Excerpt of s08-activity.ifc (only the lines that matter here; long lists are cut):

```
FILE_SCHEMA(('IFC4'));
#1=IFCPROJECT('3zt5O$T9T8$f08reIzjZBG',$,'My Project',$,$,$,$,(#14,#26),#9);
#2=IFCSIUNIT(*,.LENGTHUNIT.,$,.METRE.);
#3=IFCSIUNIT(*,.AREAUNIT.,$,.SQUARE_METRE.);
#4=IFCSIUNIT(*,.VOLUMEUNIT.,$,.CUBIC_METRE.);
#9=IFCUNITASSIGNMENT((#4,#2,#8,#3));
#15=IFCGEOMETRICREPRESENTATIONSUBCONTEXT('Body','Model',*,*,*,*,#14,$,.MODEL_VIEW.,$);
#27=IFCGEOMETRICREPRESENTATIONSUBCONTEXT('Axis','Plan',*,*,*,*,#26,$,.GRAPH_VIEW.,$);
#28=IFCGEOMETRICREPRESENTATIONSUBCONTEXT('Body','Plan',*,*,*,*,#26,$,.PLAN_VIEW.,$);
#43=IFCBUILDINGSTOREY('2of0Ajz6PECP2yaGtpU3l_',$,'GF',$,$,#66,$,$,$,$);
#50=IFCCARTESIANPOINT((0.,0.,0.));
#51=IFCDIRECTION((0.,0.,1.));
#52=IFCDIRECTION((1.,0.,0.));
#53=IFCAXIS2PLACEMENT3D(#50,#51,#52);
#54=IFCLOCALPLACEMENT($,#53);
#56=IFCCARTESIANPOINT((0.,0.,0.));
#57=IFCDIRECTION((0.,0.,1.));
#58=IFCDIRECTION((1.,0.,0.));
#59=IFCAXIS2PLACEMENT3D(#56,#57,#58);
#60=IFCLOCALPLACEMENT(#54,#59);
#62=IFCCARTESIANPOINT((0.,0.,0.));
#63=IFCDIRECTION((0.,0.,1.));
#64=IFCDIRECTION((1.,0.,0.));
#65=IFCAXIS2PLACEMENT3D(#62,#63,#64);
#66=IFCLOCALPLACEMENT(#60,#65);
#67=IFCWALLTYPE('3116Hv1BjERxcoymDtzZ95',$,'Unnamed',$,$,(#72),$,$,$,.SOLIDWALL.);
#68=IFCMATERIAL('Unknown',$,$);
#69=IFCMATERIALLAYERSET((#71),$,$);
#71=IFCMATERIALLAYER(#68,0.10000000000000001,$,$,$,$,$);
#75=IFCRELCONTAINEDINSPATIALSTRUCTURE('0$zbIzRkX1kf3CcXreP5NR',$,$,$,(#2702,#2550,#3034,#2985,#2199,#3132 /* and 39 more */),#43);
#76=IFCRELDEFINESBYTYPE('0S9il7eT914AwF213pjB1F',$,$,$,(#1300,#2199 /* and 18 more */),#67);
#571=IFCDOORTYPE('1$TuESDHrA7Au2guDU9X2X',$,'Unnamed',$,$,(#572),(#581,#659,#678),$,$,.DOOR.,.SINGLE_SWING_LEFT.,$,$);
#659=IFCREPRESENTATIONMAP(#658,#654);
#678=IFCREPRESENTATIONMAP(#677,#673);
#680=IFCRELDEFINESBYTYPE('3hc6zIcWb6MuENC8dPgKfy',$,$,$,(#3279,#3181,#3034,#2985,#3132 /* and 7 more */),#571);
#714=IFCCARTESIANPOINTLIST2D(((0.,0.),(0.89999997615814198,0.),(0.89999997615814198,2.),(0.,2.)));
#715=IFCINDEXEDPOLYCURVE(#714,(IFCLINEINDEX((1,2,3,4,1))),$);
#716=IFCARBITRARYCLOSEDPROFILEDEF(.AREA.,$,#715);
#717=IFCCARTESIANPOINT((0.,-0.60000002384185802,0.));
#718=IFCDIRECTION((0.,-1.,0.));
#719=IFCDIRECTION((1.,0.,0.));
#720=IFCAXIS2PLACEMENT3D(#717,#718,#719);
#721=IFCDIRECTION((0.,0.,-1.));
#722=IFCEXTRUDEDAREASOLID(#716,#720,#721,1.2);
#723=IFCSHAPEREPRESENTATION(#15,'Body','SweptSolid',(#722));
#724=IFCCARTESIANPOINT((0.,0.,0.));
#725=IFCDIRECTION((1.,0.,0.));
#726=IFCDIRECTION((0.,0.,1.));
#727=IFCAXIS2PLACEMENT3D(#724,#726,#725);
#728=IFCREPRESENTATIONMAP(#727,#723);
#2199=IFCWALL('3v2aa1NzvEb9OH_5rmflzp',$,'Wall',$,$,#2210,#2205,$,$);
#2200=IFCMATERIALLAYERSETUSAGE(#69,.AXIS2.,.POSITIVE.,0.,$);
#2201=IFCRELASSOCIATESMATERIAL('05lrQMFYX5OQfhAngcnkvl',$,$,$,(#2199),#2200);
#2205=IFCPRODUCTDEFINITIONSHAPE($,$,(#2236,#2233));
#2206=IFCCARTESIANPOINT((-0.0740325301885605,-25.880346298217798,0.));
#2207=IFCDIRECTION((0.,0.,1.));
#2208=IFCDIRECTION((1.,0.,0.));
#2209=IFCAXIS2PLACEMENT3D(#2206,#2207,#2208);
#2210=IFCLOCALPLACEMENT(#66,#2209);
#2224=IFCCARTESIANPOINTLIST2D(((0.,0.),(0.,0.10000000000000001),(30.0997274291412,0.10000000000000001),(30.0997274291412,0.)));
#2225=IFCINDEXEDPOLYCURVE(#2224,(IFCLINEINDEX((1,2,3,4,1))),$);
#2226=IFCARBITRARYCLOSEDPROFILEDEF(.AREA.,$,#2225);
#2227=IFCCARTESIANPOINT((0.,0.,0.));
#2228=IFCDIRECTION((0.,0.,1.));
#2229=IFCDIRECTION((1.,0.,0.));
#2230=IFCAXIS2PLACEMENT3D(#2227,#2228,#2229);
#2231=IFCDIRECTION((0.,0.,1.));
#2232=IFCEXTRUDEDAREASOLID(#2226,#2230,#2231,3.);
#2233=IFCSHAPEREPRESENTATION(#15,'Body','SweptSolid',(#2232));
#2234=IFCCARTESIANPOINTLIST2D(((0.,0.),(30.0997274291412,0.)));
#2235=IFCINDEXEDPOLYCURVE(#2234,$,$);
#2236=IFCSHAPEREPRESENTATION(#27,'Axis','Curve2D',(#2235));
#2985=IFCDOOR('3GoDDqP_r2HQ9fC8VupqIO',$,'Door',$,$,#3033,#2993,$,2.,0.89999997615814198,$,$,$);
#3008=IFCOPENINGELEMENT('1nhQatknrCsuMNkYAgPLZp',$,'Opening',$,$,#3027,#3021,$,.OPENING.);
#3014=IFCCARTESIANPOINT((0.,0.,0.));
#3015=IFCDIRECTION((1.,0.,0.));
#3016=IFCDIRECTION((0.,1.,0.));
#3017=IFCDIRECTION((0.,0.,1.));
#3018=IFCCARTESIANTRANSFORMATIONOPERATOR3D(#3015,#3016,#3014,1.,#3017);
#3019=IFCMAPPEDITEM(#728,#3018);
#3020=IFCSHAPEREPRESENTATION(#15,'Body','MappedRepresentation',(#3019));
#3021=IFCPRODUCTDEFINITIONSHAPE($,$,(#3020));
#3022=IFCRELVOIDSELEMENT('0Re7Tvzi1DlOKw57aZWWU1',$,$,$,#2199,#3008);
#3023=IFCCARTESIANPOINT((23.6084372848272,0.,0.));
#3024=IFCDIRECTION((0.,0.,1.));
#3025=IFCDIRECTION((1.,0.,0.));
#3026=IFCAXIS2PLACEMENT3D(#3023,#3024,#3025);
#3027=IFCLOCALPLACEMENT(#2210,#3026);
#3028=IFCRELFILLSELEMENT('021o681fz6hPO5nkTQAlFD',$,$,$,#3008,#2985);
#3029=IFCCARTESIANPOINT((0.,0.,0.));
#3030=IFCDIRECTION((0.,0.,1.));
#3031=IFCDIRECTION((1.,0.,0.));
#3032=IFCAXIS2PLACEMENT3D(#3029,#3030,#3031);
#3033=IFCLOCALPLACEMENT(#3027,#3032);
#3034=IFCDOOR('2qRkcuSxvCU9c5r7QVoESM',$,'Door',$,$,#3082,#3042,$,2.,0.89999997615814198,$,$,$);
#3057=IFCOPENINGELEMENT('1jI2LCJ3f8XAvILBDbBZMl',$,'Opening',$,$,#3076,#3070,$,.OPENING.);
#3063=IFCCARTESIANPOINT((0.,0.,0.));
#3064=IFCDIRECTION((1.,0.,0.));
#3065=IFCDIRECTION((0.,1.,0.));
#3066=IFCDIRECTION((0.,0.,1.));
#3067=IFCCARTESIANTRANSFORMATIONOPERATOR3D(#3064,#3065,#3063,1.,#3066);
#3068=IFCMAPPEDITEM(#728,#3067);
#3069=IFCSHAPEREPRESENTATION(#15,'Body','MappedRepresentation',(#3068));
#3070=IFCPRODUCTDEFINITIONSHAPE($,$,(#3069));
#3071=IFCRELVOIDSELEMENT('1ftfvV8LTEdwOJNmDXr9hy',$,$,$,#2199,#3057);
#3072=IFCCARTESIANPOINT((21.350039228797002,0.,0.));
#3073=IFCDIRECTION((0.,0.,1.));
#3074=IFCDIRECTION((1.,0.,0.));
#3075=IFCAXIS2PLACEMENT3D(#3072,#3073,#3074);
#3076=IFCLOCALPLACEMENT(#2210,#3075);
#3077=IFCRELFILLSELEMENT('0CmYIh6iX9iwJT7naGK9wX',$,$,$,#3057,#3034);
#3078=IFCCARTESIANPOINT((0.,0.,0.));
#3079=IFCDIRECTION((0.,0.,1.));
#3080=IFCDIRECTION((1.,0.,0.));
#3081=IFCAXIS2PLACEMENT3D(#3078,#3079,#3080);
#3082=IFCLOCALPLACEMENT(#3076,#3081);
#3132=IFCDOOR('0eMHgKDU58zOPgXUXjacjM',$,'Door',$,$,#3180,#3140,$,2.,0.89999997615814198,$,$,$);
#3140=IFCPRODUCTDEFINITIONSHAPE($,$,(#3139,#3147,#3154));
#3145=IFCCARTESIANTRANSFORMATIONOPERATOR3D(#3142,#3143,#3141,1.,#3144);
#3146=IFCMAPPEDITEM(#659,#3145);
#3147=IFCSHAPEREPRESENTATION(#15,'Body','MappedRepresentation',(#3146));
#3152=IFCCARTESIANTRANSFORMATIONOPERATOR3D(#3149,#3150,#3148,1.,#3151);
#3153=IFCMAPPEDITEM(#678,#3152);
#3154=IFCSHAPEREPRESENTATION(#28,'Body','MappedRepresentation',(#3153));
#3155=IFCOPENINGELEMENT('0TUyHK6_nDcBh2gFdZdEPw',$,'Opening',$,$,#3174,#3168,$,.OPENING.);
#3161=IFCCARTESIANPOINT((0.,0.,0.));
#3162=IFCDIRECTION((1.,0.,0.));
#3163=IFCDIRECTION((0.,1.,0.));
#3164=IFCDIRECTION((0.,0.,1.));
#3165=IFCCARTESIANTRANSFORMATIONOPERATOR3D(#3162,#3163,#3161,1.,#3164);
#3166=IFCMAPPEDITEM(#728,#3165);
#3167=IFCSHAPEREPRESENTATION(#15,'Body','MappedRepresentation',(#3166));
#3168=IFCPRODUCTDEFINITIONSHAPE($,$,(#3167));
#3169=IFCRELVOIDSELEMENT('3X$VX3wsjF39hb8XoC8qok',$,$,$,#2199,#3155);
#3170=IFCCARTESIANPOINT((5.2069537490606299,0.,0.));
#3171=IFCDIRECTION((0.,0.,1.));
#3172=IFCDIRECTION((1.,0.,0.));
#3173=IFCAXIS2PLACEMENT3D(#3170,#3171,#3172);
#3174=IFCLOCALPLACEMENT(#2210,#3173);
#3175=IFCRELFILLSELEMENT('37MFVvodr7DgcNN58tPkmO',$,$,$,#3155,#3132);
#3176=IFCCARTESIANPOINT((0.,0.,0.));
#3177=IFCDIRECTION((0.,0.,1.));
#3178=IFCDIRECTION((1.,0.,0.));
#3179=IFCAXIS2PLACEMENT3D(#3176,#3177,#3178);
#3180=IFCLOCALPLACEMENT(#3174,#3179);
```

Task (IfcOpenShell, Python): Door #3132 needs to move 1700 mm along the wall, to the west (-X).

```python
import ifcopenshell
import ifcopenshell.api.geometry
import ifcopenshell.util.placement
import ifcopenshell.util.unit

model = ifcopenshell.open("s08-activity.ifc")
unit_scale = ifcopenshell.util.unit.calculate_unit_scale(model)

door = model.by_guid("0eMHgKDU58zOPgXUXjacjM")
opening = door.FillsVoids[0].RelatingOpeningElement
wall = opening.VoidsElements[0].RelatingBuildingElement

wall_matrix = ifcopenshell.util.placement.get_local_placement(wall.ObjectPlacement)
shift = wall_matrix[:3, 0] * -1.7 / unit_scale
before = ifcopenshell.util.placement.get_local_placement(door.ObjectPlacement)[:3, 3].copy()

# The door is placed relative to its opening, so it follows when the opening moves.
matrix = ifcopenshell.util.placement.get_local_placement(opening.ObjectPlacement)
matrix[:3, 3] += shift
ifcopenshell.api.geometry.edit_object_placement(
    model, product=opening, matrix=matrix, is_si=False, should_transform_children=True
)

after = ifcopenshell.util.placement.get_local_placement(door.ObjectPlacement)[:3, 3]
print("door moved by", (after - before).round(3) + 0.0)

model.write("s08-activity_rev.ifc")
```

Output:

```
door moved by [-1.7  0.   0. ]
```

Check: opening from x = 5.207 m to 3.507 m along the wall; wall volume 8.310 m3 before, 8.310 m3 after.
